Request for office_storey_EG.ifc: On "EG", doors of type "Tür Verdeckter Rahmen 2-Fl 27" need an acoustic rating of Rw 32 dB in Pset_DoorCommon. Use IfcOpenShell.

First a look at what the model holds.

```python
import ifcopenshell
import ifcopenshell.util.element

model = ifcopenshell.open("office_storey_EG.ifc")
print(model.schema)
storey = next(s for s in model.by_type("IfcBuildingStorey") if s.Name == "EG")
doors = [e for e in ifcopenshell.util.element.get_decomposition(storey) if e.is_a("IfcDoor")]
seen = {}
for e in doors:
    element_type = ifcopenshell.util.element.get_type(e)
    key = (element_type.Name if element_type != e and element_type else None, ifcopenshell.util.element.get_pset(e, "Pset_DoorCommon", "AcousticRating"))
    seen[key] = seen.get(key, 0) + 1
for (name, value), count in sorted(seen.items(), key=str):
    print(count, "x", name, "|", value)
```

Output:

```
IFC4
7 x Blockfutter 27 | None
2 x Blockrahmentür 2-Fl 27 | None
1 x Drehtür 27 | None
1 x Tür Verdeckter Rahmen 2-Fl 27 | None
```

```python
import ifcopenshell
import ifcopenshell.api.pset
import ifcopenshell.util.element

model = ifcopenshell.open("office_storey_EG.ifc")

storey = next(s for s in model.by_type("IfcBuildingStorey") if s.Name == "EG")
doors = [e for e in ifcopenshell.util.element.get_decomposition(storey) if e.is_a("IfcDoor")]

count = 0
for e in doors:
    element_type = ifcopenshell.util.element.get_type(e)
    if element_type in (None, e) or element_type.Name != "Tür Verdeckter Rahmen 2-Fl 27":
        continue
    # add_pset returns the element's existing set when there is one.
    pset = ifcopenshell.api.pset.add_pset(model, product=e, name="Pset_DoorCommon")
    ifcopenshell.api.pset.edit_pset(model, pset=pset, properties={"AcousticRating": "Rw 32 dB"})
    count += 1

print(count, "doors updated")

model.write("office_storey_EG_updated.ifc")
```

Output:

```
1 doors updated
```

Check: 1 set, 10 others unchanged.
